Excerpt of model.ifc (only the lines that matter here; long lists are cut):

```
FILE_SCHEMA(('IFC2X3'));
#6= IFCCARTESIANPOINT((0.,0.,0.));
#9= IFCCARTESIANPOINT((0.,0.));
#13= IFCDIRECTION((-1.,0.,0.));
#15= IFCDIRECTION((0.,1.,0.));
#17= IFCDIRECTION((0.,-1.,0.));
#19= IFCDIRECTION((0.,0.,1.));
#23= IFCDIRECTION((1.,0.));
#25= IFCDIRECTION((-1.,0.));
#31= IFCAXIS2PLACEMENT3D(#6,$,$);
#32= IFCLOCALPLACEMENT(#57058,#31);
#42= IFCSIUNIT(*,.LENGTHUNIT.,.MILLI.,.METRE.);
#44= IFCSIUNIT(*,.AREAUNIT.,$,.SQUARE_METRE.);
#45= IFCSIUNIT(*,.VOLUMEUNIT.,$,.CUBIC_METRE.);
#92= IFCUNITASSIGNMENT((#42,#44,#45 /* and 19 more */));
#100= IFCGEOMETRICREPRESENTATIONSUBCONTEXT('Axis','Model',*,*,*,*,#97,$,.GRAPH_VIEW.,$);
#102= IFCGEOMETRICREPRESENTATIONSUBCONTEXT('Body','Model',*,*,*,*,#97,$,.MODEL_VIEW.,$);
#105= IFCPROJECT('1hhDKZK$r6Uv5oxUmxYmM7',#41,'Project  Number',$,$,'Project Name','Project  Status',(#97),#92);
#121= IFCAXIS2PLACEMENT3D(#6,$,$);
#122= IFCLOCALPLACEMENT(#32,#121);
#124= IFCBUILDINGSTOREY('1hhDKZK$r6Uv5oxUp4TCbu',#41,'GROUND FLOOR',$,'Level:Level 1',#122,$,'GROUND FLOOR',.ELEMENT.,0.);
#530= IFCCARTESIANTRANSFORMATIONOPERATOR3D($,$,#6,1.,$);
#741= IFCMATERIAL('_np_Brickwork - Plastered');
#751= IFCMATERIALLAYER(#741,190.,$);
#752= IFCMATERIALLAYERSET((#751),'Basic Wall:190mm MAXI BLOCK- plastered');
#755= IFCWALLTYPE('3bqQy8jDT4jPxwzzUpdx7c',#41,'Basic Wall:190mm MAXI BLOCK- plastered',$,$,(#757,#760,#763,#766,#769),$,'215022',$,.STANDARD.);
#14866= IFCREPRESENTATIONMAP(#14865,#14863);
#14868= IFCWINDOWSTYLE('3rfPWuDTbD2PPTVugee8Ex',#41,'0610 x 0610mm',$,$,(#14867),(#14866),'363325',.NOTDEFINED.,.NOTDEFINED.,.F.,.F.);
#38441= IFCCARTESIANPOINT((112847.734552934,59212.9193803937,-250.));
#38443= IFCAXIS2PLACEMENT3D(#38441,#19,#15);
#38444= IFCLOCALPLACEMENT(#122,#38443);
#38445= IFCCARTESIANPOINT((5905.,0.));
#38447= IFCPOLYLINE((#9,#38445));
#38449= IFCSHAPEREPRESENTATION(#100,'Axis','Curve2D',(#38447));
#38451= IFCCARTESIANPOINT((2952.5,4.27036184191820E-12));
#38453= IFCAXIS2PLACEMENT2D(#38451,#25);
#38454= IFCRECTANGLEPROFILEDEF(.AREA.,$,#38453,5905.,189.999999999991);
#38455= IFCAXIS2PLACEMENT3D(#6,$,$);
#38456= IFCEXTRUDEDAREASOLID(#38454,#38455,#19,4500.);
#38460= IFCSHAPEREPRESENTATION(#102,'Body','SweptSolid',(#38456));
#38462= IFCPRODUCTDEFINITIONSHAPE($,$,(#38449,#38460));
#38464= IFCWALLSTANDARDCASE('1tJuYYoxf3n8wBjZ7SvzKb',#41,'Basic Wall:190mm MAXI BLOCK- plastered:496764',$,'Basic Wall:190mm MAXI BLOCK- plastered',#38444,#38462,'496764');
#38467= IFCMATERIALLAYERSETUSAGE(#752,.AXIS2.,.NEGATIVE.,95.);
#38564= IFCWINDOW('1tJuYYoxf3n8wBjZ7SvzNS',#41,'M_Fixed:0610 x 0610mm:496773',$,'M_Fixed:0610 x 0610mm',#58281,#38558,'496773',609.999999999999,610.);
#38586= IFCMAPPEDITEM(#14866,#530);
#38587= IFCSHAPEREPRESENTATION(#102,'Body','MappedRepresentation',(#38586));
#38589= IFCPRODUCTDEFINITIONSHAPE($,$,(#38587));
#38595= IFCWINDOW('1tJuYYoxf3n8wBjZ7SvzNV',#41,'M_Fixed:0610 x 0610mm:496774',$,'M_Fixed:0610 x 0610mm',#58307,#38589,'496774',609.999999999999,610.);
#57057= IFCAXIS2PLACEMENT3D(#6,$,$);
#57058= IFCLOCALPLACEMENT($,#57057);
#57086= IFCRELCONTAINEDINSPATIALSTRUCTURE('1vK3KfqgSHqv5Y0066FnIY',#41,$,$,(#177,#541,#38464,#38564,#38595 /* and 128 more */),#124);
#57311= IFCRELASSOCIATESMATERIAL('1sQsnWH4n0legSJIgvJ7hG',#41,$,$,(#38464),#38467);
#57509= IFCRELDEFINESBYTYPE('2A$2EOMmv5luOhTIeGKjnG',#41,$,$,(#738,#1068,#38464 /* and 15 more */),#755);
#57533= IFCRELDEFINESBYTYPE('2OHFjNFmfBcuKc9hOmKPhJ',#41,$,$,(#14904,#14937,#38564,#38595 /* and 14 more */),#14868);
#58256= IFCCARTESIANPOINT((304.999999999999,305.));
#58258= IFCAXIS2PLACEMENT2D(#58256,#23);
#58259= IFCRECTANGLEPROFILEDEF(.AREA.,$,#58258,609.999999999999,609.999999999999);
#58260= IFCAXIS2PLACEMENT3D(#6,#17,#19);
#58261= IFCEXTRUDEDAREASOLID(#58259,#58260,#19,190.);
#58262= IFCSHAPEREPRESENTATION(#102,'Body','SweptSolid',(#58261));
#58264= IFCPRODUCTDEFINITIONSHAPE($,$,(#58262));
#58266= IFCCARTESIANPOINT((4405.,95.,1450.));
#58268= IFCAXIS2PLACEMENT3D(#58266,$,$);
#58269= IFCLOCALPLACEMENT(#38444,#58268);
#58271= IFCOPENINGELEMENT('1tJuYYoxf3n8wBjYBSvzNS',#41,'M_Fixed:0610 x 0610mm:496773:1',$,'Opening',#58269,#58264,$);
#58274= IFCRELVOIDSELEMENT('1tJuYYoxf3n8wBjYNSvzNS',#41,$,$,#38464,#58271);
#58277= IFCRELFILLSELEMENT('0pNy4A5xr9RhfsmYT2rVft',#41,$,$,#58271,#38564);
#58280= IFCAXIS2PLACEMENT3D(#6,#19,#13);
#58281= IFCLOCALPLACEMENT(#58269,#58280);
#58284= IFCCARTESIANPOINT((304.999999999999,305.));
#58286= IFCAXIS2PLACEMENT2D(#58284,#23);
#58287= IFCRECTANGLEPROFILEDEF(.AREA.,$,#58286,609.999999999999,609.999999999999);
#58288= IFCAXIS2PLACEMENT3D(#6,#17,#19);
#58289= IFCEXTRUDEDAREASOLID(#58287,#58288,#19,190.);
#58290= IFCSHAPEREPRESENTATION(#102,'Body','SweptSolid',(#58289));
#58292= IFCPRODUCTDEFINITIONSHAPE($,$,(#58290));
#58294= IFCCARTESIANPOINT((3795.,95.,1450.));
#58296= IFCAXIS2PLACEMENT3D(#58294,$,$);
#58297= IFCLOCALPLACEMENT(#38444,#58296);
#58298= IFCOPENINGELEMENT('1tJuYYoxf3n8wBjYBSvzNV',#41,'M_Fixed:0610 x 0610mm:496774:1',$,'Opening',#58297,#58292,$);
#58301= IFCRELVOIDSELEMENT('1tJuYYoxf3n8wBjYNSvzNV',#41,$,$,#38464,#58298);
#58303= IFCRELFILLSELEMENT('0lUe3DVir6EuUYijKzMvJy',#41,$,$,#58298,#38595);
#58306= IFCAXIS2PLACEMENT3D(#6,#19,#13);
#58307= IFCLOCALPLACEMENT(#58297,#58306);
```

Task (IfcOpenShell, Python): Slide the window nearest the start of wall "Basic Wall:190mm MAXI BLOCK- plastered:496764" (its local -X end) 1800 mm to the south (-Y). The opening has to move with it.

```python
import ifcopenshell
import ifcopenshell.api.geometry
import ifcopenshell.util.placement
import ifcopenshell.util.unit

model = ifcopenshell.open("model.ifc")
unit_scale = ifcopenshell.util.unit.calculate_unit_scale(model)

window = model.by_guid("1tJuYYoxf3n8wBjZ7SvzNV")
opening = window.FillsVoids[0].RelatingOpeningElement
wall = opening.VoidsElements[0].RelatingBuildingElement

wall_matrix = ifcopenshell.util.placement.get_local_placement(wall.ObjectPlacement)
shift = wall_matrix[:3, 0] * -1.8 / unit_scale
before = ifcopenshell.util.placement.get_local_placement(window.ObjectPlacement)[:3, 3].copy()

# The window is placed relative to its opening, so it follows when the opening moves.
matrix = ifcopenshell.util.placement.get_local_placement(opening.ObjectPlacement)
matrix[:3, 3] += shift
ifcopenshell.api.geometry.edit_object_placement(
    model, product=opening, matrix=matrix, is_si=False, should_transform_children=True
)

after = ifcopenshell.util.placement.get_local_placement(window.ObjectPlacement)[:3, 3]
print("window moved by", (after - before).round(3) + 0.0)

model.write("model_v2.ifc")
```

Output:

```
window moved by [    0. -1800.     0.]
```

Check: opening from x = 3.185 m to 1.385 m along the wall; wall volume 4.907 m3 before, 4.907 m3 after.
